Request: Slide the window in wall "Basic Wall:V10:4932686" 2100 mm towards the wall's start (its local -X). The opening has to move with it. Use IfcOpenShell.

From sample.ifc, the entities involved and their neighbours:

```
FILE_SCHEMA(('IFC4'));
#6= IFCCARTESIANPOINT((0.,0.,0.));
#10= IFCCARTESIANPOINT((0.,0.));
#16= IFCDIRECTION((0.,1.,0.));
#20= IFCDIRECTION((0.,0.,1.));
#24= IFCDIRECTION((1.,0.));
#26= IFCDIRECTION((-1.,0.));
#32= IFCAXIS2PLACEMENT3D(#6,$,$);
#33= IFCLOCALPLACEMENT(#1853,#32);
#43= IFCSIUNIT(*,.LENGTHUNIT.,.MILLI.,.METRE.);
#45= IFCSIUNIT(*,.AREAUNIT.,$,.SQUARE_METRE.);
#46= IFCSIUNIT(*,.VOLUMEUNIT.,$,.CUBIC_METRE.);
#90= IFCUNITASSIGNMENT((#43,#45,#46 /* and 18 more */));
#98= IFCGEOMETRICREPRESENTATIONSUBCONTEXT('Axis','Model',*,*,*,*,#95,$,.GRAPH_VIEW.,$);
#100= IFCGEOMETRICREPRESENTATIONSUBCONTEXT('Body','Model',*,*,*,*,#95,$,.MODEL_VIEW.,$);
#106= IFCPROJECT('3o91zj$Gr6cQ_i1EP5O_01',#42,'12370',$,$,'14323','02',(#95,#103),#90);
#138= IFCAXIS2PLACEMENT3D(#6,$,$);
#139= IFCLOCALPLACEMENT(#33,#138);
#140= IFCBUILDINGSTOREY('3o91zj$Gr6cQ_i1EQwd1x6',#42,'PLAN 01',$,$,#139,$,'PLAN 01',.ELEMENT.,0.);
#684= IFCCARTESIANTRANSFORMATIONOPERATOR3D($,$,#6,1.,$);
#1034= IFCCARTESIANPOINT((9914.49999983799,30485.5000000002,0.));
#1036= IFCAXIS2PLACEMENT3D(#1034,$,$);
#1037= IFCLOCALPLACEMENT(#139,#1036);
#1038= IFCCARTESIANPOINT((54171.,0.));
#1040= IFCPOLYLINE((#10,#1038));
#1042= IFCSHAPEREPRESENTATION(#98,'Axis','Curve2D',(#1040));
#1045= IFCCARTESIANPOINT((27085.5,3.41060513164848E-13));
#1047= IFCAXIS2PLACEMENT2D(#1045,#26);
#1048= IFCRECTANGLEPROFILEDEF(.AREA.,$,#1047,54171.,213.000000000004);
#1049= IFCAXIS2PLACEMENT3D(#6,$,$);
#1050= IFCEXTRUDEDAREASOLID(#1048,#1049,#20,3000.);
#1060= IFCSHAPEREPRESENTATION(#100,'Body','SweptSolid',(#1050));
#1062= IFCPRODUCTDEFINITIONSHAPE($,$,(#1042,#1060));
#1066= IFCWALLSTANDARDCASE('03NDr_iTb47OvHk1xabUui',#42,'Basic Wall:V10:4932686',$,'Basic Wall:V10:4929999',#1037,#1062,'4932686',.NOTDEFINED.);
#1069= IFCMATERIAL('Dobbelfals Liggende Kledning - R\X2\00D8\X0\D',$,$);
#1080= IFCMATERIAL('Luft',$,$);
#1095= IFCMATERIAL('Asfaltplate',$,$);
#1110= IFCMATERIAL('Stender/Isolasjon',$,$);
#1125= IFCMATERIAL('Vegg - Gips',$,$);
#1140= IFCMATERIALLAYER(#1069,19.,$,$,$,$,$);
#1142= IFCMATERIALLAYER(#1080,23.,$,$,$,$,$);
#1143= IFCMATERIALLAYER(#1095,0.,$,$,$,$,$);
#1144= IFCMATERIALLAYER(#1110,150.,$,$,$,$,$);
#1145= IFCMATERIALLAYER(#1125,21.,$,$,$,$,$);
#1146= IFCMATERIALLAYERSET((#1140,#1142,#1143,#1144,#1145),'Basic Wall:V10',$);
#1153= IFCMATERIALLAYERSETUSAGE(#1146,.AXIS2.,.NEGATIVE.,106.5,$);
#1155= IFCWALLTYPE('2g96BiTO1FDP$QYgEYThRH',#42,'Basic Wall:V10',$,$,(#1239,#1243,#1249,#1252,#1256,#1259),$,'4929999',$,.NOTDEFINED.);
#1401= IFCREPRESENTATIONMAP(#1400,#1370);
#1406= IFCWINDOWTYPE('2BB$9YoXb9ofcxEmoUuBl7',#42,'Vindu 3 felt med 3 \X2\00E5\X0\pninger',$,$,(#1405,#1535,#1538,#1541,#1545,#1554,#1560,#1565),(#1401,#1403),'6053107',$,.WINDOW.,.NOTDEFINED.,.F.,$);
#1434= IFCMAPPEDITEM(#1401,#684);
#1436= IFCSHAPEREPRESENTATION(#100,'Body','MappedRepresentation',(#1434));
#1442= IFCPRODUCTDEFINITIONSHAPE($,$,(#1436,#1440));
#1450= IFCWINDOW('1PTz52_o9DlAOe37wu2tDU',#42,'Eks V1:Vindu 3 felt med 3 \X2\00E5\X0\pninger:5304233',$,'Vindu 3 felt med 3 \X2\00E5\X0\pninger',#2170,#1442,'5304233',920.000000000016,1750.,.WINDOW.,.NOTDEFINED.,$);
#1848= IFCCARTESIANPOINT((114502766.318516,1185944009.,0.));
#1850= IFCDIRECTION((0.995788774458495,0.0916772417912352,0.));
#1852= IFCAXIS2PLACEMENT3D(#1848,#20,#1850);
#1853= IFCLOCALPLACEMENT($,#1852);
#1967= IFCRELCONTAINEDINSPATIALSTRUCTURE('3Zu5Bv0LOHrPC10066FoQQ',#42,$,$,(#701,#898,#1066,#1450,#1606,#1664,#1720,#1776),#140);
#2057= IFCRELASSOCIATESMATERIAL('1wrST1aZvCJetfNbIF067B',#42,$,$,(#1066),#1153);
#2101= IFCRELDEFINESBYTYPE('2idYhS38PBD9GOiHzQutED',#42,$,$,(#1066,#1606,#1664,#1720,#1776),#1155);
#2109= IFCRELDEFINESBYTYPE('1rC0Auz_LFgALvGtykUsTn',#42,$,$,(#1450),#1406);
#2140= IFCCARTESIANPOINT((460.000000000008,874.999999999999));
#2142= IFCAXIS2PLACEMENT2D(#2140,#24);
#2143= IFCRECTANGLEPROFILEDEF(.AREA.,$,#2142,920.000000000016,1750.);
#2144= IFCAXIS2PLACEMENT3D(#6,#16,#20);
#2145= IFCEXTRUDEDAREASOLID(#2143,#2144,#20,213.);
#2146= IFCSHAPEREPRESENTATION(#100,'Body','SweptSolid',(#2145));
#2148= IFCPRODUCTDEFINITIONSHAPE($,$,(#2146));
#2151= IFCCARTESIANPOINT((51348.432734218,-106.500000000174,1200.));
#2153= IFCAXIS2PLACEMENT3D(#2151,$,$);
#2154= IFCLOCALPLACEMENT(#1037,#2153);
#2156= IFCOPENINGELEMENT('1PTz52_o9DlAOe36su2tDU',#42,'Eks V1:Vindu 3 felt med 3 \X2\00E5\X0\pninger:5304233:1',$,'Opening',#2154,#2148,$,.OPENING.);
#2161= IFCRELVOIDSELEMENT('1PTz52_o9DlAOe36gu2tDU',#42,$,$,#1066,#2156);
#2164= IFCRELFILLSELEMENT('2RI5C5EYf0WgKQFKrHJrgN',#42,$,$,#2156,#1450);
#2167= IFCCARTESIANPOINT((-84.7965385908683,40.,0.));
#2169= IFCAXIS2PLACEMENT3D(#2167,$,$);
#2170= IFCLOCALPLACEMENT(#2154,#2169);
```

```python
import ifcopenshell
import ifcopenshell.api.geometry
import ifcopenshell.util.placement
import ifcopenshell.util.unit

model = ifcopenshell.open("sample.ifc")
unit_scale = ifcopenshell.util.unit.calculate_unit_scale(model)

window = model.by_guid("1PTz52_o9DlAOe37wu2tDU")
opening = window.FillsVoids[0].RelatingOpeningElement
wall = opening.VoidsElements[0].RelatingBuildingElement

wall_matrix = ifcopenshell.util.placement.get_local_placement(wall.ObjectPlacement)
shift = wall_matrix[:3, 0] * -2.1 / unit_scale
before = ifcopenshell.util.placement.get_local_placement(window.ObjectPlacement)[:3, 3].copy()

# The window is placed relative to its opening, so it follows when the opening moves.
matrix = ifcopenshell.util.placement.get_local_placement(opening.ObjectPlacement)
matrix[:3, 3] += shift
ifcopenshell.api.geometry.edit_object_placement(
    model, product=opening, matrix=matrix, is_si=False, should_transform_children=True
)

after = ifcopenshell.util.placement.get_local_placement(window.ObjectPlacement)[:3, 3]
print("window moved by", (after - before).round(3) + 0.0)

model.write("sample_rev.ifc")
```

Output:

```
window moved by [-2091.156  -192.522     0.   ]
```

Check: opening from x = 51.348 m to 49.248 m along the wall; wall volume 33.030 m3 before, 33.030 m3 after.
